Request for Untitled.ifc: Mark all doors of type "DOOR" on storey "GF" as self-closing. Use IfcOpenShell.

First a look at what the model holds.

```python
import ifcopenshell
import ifcopenshell.util.element

model = ifcopenshell.open("Untitled.ifc")
print(model.schema)
storey = next(s for s in model.by_type("IfcBuildingStorey") if s.Name == "GF")
doors = [e for e in ifcopenshell.util.element.get_decomposition(storey) if e.is_a("IfcDoor")]
seen = {}
for e in doors:
    element_type = ifcopenshell.util.element.get_type(e)
    key = (element_type.Name if element_type != e and element_type else None, ifcopenshell.util.element.get_pset(e, "Pset_DoorCommon", "SelfClosing"))
    seen[key] = seen.get(key, 0) + 1
for (name, value), count in sorted(seen.items(), key=str):
    print(count, "x", name, "|", value)
```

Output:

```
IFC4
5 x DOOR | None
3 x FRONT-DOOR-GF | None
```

```python
import ifcopenshell
import ifcopenshell.api.pset
import ifcopenshell.util.element

model = ifcopenshell.open("Untitled.ifc")

storey = next(s for s in model.by_type("IfcBuildingStorey") if s.Name == "GF")
doors = [e for e in ifcopenshell.util.element.get_decomposition(storey) if e.is_a("IfcDoor")]

count = 0
for e in doors:
    element_type = ifcopenshell.util.element.get_type(e)
    if element_type in (None, e) or element_type.Name != "DOOR":
        continue
    # add_pset returns the element's existing set when there is one.
    pset = ifcopenshell.api.pset.add_pset(model, product=e, name="Pset_DoorCommon")
    ifcopenshell.api.pset.edit_pset(model, pset=pset, properties={"SelfClosing": True})
    count += 1

print(count, "doors updated")

model.write("Untitled_updated.ifc")
```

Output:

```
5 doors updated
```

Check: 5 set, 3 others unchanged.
